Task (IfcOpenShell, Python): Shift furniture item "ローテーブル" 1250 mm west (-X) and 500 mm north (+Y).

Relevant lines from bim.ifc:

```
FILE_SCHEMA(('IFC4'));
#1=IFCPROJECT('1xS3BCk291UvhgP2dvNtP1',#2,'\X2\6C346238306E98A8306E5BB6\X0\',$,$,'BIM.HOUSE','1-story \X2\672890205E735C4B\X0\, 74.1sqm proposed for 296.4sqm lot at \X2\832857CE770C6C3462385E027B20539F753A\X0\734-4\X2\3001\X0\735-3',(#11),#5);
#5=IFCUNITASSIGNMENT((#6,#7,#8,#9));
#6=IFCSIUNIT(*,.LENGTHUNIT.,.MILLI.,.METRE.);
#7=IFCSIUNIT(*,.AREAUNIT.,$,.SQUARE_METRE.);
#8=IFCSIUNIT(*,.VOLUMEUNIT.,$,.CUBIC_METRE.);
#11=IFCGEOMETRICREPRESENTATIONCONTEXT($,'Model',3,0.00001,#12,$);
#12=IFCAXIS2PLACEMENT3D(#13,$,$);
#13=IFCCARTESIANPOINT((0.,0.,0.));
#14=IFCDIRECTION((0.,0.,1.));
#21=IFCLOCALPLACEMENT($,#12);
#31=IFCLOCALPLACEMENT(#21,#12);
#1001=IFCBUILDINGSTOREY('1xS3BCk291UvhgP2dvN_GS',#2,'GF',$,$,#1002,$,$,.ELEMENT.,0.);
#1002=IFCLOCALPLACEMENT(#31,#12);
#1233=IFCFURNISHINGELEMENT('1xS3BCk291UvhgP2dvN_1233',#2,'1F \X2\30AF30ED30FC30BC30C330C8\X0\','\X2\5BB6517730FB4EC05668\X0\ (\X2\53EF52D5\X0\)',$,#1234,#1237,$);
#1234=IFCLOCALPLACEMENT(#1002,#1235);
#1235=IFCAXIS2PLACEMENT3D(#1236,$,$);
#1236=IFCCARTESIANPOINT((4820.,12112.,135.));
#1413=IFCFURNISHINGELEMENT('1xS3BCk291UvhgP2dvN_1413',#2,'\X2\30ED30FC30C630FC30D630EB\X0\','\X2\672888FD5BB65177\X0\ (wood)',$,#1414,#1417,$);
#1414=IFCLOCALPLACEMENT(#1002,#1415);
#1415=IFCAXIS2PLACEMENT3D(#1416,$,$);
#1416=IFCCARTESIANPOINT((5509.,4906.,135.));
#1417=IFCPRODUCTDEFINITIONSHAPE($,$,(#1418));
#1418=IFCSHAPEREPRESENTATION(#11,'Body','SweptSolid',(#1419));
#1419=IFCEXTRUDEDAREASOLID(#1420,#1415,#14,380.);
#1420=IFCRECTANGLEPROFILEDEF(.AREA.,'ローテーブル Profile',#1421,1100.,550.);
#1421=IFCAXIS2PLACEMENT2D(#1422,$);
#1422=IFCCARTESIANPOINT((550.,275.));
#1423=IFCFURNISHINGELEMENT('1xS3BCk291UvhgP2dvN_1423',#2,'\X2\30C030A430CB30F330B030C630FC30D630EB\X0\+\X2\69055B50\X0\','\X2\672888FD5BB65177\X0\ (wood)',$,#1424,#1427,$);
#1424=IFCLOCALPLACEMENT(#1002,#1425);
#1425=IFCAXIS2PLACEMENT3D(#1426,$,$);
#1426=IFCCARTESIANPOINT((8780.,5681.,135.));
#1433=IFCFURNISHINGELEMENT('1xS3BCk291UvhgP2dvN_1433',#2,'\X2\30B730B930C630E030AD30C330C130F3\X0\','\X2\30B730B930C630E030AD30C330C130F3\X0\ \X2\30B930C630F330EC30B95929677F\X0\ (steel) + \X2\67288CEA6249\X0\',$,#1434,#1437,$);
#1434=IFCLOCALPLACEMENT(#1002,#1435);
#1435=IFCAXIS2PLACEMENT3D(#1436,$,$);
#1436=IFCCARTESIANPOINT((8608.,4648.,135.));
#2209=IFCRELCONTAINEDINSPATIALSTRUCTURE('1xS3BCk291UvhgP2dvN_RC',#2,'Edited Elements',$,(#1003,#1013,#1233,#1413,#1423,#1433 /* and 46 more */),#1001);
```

```python
import ifcopenshell
import ifcopenshell.api.geometry
import ifcopenshell.util.placement

model = ifcopenshell.open("bim.ifc")

item = model.by_guid("1xS3BCk291UvhgP2dvN_1413")
matrix = ifcopenshell.util.placement.get_local_placement(item.ObjectPlacement)
matrix[0, 3] -= 1250.0
matrix[1, 3] += 500.0
ifcopenshell.api.geometry.edit_object_placement(model, product=item, matrix=matrix, is_si=False)

print(ifcopenshell.util.placement.get_local_placement(item.ObjectPlacement).round(3) + 0.0)

model.write("bim-out.ifc")
```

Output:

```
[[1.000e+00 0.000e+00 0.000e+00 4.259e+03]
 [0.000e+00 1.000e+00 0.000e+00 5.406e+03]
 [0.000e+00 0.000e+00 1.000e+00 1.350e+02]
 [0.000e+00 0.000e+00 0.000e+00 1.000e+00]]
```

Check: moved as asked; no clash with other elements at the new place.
